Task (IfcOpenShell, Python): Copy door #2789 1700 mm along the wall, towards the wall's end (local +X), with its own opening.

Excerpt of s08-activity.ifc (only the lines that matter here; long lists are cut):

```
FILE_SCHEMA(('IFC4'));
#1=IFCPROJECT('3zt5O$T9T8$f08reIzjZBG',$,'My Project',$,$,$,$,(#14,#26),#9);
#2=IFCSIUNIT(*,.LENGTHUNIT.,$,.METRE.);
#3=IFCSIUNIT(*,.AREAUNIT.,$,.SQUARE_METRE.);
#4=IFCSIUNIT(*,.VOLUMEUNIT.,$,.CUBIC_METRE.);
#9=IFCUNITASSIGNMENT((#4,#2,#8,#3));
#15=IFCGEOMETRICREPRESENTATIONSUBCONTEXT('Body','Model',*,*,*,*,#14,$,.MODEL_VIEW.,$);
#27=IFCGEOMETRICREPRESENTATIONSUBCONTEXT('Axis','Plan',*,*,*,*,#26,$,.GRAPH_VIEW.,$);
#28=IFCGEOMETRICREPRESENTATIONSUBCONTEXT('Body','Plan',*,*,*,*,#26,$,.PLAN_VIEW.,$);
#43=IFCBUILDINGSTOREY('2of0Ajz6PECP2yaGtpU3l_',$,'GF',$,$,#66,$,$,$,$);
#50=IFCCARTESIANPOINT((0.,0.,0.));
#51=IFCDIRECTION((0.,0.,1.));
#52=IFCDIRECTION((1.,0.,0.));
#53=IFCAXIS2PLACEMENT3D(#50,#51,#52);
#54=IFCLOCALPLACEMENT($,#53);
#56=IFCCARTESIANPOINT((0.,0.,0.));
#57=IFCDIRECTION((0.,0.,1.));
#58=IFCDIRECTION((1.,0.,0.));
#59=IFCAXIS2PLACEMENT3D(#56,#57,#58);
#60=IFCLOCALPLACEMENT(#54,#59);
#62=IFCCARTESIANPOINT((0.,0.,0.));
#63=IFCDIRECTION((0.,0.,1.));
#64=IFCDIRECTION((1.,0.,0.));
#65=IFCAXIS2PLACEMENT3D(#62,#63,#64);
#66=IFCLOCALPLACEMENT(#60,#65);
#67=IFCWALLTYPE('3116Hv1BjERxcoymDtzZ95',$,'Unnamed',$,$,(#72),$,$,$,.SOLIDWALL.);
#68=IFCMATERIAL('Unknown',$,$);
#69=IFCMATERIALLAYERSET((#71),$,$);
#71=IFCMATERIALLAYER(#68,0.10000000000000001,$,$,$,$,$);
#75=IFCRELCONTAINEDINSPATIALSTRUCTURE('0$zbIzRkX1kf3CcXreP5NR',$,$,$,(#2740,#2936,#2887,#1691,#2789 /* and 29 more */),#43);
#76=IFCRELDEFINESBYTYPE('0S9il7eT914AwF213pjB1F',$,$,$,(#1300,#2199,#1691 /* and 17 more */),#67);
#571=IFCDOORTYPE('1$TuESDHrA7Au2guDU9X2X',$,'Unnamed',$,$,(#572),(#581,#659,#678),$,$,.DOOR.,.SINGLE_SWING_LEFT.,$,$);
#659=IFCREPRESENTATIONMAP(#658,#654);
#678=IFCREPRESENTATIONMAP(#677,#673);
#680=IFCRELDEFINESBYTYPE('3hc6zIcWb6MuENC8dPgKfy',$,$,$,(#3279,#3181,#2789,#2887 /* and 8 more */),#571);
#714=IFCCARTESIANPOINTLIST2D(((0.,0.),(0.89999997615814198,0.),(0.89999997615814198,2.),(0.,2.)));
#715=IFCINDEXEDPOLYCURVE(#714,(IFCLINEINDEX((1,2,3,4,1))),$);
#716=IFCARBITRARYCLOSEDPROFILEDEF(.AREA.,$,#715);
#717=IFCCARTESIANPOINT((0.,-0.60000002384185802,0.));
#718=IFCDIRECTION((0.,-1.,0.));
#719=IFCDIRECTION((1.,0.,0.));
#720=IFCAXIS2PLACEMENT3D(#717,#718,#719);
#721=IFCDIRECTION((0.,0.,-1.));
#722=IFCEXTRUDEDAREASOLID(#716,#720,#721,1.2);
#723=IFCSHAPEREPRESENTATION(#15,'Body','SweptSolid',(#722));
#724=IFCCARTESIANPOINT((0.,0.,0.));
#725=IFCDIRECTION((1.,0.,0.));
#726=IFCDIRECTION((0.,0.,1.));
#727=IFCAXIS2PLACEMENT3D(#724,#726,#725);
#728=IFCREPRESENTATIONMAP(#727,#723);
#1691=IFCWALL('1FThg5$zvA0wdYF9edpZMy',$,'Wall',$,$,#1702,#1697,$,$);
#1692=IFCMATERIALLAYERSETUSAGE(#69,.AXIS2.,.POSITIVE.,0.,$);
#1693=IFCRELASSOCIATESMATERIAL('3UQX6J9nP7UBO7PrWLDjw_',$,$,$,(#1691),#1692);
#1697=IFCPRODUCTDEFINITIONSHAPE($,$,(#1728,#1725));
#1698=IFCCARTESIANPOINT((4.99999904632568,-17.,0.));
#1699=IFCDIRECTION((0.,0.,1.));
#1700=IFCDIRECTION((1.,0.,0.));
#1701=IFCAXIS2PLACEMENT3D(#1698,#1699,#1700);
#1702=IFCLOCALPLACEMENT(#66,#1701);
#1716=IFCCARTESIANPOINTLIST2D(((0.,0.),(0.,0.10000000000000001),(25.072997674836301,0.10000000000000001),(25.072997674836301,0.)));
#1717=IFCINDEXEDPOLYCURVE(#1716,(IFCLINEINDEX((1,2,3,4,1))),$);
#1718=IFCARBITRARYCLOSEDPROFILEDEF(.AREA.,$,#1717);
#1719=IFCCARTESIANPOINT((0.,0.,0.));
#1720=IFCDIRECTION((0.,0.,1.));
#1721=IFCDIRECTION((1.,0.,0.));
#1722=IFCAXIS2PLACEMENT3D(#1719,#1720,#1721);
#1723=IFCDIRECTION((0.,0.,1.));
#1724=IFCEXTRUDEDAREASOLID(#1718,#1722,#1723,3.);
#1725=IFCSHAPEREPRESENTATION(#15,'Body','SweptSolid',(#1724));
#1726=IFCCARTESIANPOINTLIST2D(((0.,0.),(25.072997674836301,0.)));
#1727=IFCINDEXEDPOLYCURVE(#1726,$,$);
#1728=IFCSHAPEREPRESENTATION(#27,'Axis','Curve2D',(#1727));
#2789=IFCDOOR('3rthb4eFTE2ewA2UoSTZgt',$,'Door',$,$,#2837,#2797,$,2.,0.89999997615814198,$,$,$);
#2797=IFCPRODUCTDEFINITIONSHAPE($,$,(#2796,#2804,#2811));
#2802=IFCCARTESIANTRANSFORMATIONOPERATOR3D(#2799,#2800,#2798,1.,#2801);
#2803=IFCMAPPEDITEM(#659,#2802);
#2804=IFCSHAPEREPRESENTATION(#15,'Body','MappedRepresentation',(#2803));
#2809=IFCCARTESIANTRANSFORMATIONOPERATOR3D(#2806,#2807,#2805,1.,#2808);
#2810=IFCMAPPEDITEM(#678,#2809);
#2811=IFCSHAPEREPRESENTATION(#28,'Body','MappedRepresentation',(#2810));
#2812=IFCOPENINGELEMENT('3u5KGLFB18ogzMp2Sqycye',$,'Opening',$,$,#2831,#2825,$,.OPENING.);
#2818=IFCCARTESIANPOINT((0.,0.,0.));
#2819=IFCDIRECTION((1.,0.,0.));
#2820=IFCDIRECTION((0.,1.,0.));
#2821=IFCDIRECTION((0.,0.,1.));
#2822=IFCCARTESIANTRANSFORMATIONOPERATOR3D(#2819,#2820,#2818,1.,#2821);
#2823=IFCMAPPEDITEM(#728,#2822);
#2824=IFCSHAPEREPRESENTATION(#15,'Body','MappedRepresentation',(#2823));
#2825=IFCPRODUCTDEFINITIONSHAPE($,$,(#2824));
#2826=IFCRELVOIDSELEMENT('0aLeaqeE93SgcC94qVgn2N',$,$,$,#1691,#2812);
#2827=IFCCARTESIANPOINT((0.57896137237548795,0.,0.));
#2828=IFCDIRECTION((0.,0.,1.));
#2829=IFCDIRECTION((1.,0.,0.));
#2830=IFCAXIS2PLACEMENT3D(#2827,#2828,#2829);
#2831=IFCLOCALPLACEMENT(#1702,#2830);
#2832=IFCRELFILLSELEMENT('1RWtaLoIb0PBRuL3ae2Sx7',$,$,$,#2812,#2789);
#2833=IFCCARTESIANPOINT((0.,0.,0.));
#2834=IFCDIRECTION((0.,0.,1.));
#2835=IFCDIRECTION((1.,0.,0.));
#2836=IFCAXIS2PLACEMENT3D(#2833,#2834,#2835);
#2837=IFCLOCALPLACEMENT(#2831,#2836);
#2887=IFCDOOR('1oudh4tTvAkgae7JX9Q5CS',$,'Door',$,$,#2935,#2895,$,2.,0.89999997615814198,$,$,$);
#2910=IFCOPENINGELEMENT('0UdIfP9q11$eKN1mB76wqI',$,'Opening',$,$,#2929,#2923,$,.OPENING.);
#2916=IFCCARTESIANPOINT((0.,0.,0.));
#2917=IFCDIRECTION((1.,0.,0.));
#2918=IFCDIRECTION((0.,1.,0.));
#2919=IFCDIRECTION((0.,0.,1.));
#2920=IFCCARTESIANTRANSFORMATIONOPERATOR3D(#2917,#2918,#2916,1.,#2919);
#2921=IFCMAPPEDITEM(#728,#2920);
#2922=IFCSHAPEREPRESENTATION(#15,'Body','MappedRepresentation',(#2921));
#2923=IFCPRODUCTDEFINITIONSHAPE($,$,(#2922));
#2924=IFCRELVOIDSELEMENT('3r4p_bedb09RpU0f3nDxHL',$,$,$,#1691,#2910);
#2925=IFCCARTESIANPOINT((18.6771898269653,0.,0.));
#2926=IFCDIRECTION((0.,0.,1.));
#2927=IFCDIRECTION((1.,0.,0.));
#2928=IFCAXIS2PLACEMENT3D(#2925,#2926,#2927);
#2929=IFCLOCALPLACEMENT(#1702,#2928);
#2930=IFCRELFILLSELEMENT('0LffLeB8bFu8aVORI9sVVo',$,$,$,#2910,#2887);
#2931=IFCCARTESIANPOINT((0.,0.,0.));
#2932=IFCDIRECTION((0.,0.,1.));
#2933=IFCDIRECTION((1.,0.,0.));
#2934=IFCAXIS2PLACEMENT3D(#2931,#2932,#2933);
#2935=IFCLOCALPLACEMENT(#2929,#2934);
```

```python
import ifcopenshell
import ifcopenshell.api.feature
import ifcopenshell.api.geometry
import ifcopenshell.api.root
import ifcopenshell.geom
import ifcopenshell.util.element
import ifcopenshell.util.placement
import ifcopenshell.util.shape

model = ifcopenshell.open("s08-activity.ifc")
settings = ifcopenshell.geom.settings()


def volume(element):
    """Net volume in cubic metres, openings subtracted."""
    shape = ifcopenshell.geom.create_shape(settings, element)
    return ifcopenshell.util.shape.get_volume(shape.geometry)


door = model.by_guid("3rthb4eFTE2ewA2UoSTZgt")
opening = door.FillsVoids[0].RelatingOpeningElement
wall = opening.VoidsElements[0].RelatingBuildingElement
before = volume(wall)
shift = ifcopenshell.util.placement.get_local_placement(wall.ObjectPlacement)[:3, 0] * 1.7

# copy_class copies the void relationship, type, container and properties, but no geometry.
new_opening = ifcopenshell.api.root.copy_class(model, product=opening)
new_opening.Representation = ifcopenshell.util.element.copy_deep(
    model, opening.Representation, exclude=["IfcGeometricRepresentationContext", "IfcRepresentationMap"]
)
new_door = ifcopenshell.api.root.copy_class(model, product=door)
new_door.Representation = ifcopenshell.util.element.copy_deep(
    model, door.Representation, exclude=["IfcGeometricRepresentationContext", "IfcRepresentationMap"]
)
ifcopenshell.api.feature.add_filling(model, opening=new_opening, element=new_door)

for old, new in ((opening, new_opening), (door, new_door)):
    matrix = ifcopenshell.util.placement.get_local_placement(old.ObjectPlacement)
    matrix[:3, 3] += shift
    ifcopenshell.api.geometry.edit_object_placement(model, product=new, matrix=matrix, is_si=False)

after = volume(wall)

print(f"wall volume {before:.3f} -> {after:.3f} m3")

model.write("s08-activity_v2.ifc")
```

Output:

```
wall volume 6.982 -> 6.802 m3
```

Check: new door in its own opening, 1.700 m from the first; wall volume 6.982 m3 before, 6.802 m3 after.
